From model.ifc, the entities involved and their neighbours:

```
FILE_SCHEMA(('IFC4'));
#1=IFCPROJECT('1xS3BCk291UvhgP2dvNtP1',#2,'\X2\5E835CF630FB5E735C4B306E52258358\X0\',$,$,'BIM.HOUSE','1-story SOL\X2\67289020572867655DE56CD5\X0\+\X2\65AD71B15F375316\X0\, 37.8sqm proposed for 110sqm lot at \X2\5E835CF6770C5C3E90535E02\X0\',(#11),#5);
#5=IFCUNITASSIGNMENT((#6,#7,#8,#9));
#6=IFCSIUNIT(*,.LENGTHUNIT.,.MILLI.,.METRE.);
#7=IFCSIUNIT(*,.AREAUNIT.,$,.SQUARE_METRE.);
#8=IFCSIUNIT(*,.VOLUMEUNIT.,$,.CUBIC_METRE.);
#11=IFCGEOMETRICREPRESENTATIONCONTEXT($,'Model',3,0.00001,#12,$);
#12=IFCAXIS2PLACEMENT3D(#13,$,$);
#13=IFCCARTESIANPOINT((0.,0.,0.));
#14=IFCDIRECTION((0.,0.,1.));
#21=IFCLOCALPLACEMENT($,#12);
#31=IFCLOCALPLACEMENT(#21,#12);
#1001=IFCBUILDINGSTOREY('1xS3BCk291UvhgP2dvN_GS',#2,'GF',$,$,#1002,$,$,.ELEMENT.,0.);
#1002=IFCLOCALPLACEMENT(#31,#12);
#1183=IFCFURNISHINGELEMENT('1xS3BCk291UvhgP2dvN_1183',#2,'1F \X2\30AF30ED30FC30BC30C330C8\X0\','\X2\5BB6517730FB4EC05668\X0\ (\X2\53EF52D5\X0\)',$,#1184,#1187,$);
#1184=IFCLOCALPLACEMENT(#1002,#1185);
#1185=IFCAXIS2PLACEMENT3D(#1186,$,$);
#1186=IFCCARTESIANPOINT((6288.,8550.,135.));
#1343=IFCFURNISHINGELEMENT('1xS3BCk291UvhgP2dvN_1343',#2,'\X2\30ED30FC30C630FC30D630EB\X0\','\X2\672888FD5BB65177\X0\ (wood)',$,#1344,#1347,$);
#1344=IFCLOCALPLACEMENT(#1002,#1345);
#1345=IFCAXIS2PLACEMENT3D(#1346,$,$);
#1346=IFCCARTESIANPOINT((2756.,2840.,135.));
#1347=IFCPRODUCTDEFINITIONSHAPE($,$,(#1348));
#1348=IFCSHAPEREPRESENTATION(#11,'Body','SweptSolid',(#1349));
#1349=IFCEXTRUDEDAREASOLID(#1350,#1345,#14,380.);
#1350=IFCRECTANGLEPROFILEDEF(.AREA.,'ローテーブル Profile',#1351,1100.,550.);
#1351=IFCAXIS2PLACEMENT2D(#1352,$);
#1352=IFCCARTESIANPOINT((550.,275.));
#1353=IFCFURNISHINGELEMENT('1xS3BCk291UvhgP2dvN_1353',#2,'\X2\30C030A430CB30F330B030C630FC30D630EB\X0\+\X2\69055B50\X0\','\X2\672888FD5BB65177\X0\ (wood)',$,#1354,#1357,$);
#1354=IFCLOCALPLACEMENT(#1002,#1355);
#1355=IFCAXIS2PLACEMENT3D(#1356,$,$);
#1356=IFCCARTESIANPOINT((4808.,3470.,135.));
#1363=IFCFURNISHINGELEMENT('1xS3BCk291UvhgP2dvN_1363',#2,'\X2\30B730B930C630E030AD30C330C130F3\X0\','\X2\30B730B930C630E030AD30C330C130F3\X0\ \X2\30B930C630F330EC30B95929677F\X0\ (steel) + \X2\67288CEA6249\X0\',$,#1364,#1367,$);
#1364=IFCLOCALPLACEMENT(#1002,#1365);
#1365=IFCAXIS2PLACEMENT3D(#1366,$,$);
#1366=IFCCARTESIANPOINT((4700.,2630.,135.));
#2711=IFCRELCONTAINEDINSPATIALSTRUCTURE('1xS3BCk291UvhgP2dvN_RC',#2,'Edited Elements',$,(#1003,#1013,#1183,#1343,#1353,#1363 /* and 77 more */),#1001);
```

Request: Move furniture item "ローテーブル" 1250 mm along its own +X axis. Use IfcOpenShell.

```python
import ifcopenshell
import ifcopenshell.api.geometry
import ifcopenshell.util.placement
import ifcopenshell.util.unit

model = ifcopenshell.open("model.ifc")
unit_scale = ifcopenshell.util.unit.calculate_unit_scale(model)

item = model.by_guid("1xS3BCk291UvhgP2dvN_1343")
matrix = ifcopenshell.util.placement.get_local_placement(item.ObjectPlacement)
matrix[:3, 3] += matrix[:3, 0] * 1.25 / unit_scale
ifcopenshell.api.geometry.edit_object_placement(model, product=item, matrix=matrix, is_si=False)

print(ifcopenshell.util.placement.get_local_placement(item.ObjectPlacement).round(3) + 0.0)

model.write("model_v2.ifc")
```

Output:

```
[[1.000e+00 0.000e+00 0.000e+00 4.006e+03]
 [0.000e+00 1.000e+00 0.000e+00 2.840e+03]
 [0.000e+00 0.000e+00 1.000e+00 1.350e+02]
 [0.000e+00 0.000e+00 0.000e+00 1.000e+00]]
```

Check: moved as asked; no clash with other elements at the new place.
